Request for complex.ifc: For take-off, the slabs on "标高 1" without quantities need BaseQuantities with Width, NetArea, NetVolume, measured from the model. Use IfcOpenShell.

First a look at what the model holds.

```python
import ifcopenshell
import ifcopenshell.util.element
import ifcopenshell.util.unit

model = ifcopenshell.open("complex.ifc")
print(model.schema)
for unit_type in ("LENGTHUNIT", "AREAUNIT", "VOLUMEUNIT"):
    print(unit_type, ifcopenshell.util.unit.calculate_unit_scale(model, unit_type))
storey = next(s for s in model.by_type("IfcBuildingStorey") if s.Name == "标高 1")
slabs = [e for e in ifcopenshell.util.element.get_decomposition(storey) if e.is_a("IfcSlab")]
for e in sorted(slabs, key=lambda e: e.id()):
    print(e.id(), e.is_a(), e.Name, list(ifcopenshell.util.element.get_psets(e, qtos_only=True)), sep=" | ")
```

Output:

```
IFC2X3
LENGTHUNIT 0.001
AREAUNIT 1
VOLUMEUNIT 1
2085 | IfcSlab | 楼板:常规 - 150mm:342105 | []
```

```python
import ifcopenshell
import ifcopenshell.api.pset
import ifcopenshell.geom
import ifcopenshell.util.element
import ifcopenshell.util.shape
import ifcopenshell.util.unit

model = ifcopenshell.open("complex.ifc")
unit_scale = ifcopenshell.util.unit.calculate_unit_scale(model)
area_scale = ifcopenshell.util.unit.calculate_unit_scale(model, "AREAUNIT")
volume_scale = ifcopenshell.util.unit.calculate_unit_scale(model, "VOLUMEUNIT")
settings = ifcopenshell.geom.settings()

storey = next(s for s in model.by_type("IfcBuildingStorey") if s.Name == "标高 1")
slabs = [e for e in ifcopenshell.util.element.get_decomposition(storey) if e.is_a("IfcSlab")]

for e in sorted(slabs, key=lambda e: e.id()):
    if ifcopenshell.util.element.get_psets(e, qtos_only=True, should_inherit=False):
        continue
    # Geometry comes back in metres, in the element's own axes.
    shape = ifcopenshell.geom.create_shape(settings, e)
    values = {
        "Width": ifcopenshell.util.shape.get_z(shape.geometry) / unit_scale,
        "NetArea": ifcopenshell.util.shape.get_footprint_area(shape.geometry) / area_scale,
        "NetVolume": ifcopenshell.util.shape.get_volume(shape.geometry) / volume_scale,
    }
    qto = ifcopenshell.api.pset.add_qto(model, product=e, name="BaseQuantities")
    ifcopenshell.api.pset.edit_qto(model, qto=qto, properties=values)
    print(e.id(), {k: round(v, 3) for k, v in values.items()})

model.write("complex-out.ifc")
```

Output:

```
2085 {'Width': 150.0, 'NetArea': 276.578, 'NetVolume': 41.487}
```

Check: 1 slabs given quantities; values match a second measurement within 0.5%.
